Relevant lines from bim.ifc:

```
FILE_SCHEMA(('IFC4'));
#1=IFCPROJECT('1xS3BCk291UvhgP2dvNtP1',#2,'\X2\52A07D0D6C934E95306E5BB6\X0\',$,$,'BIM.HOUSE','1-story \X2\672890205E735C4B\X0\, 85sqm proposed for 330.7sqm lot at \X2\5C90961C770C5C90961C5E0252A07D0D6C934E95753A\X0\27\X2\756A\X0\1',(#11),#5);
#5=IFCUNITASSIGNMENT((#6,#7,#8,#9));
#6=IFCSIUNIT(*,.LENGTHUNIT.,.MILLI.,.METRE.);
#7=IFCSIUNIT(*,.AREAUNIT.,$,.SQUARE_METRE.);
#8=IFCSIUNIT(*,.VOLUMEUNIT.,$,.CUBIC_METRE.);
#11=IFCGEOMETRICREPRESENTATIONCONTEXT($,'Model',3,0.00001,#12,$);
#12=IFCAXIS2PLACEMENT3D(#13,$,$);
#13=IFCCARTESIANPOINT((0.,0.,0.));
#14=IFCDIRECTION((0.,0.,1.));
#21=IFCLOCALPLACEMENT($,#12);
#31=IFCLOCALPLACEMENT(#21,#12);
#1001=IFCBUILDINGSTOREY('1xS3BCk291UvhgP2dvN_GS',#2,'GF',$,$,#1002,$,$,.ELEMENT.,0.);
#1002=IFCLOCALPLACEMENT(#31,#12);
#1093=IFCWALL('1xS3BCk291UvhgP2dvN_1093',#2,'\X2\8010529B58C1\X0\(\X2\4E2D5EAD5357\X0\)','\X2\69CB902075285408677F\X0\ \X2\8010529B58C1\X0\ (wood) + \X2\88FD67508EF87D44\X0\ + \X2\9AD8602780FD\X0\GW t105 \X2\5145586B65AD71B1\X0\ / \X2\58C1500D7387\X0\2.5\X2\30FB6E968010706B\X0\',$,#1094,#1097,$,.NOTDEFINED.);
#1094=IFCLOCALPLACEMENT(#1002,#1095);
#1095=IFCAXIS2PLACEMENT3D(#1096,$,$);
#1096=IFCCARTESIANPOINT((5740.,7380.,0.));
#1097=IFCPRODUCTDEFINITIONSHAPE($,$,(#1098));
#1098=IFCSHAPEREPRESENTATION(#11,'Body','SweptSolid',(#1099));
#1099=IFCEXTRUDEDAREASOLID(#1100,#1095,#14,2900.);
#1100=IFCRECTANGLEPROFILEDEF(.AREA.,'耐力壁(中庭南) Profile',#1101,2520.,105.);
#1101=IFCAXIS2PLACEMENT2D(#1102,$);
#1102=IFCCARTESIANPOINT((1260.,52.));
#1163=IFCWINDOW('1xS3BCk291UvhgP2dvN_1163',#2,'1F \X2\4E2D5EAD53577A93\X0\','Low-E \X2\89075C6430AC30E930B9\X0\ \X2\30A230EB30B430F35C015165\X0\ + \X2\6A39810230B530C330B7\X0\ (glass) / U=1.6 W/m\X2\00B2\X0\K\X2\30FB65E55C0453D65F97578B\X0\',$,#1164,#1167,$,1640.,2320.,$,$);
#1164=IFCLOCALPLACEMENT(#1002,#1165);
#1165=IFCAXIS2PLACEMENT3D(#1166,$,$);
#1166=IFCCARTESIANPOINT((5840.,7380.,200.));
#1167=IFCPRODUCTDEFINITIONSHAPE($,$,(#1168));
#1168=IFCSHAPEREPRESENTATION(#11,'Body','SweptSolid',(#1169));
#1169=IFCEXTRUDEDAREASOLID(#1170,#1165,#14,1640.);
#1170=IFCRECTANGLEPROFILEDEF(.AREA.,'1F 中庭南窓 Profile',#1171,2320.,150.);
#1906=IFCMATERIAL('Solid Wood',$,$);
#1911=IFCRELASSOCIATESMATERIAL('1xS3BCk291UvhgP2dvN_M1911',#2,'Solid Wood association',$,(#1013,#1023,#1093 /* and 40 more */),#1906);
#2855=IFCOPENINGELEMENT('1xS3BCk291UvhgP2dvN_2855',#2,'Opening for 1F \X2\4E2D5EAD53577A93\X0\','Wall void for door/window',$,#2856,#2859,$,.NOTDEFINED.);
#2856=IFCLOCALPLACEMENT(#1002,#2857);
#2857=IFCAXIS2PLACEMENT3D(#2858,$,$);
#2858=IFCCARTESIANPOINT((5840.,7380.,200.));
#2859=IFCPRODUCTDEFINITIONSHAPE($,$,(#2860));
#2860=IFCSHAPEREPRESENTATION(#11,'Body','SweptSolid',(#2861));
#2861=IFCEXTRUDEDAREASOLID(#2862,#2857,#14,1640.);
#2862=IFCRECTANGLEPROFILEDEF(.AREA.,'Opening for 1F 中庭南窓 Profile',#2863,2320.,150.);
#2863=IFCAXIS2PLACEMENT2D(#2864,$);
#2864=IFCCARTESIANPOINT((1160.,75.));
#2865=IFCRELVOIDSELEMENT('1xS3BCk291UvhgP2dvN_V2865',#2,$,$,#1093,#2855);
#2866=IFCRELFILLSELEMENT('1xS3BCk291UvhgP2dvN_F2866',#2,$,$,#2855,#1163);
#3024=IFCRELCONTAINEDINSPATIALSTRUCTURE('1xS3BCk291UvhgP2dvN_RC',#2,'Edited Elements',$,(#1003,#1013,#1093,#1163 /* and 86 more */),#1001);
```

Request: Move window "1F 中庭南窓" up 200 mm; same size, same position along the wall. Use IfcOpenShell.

```python
import numpy as np
import ifcopenshell
import ifcopenshell.api.geometry
import ifcopenshell.util.placement
import ifcopenshell.util.unit

model = ifcopenshell.open("bim.ifc")
unit_scale = ifcopenshell.util.unit.calculate_unit_scale(model)

window = model.by_guid("1xS3BCk291UvhgP2dvN_1163")
opening = window.FillsVoids[0].RelatingOpeningElement
dz = 0.2 / unit_scale

shift = np.array([0.0, 0.0, dz])
# The window is not placed relative to its opening, so move both.
for product in (opening, window):
    matrix = ifcopenshell.util.placement.get_local_placement(product.ObjectPlacement)
    matrix[:3, 3] += shift
    ifcopenshell.api.geometry.edit_object_placement(model, product=product, matrix=matrix, is_si=False)

print(f"moved by {dz * unit_scale:+.3f} m")

model.write("bim_updated.ifc")
```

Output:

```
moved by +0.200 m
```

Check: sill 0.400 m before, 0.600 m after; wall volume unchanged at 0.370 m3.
